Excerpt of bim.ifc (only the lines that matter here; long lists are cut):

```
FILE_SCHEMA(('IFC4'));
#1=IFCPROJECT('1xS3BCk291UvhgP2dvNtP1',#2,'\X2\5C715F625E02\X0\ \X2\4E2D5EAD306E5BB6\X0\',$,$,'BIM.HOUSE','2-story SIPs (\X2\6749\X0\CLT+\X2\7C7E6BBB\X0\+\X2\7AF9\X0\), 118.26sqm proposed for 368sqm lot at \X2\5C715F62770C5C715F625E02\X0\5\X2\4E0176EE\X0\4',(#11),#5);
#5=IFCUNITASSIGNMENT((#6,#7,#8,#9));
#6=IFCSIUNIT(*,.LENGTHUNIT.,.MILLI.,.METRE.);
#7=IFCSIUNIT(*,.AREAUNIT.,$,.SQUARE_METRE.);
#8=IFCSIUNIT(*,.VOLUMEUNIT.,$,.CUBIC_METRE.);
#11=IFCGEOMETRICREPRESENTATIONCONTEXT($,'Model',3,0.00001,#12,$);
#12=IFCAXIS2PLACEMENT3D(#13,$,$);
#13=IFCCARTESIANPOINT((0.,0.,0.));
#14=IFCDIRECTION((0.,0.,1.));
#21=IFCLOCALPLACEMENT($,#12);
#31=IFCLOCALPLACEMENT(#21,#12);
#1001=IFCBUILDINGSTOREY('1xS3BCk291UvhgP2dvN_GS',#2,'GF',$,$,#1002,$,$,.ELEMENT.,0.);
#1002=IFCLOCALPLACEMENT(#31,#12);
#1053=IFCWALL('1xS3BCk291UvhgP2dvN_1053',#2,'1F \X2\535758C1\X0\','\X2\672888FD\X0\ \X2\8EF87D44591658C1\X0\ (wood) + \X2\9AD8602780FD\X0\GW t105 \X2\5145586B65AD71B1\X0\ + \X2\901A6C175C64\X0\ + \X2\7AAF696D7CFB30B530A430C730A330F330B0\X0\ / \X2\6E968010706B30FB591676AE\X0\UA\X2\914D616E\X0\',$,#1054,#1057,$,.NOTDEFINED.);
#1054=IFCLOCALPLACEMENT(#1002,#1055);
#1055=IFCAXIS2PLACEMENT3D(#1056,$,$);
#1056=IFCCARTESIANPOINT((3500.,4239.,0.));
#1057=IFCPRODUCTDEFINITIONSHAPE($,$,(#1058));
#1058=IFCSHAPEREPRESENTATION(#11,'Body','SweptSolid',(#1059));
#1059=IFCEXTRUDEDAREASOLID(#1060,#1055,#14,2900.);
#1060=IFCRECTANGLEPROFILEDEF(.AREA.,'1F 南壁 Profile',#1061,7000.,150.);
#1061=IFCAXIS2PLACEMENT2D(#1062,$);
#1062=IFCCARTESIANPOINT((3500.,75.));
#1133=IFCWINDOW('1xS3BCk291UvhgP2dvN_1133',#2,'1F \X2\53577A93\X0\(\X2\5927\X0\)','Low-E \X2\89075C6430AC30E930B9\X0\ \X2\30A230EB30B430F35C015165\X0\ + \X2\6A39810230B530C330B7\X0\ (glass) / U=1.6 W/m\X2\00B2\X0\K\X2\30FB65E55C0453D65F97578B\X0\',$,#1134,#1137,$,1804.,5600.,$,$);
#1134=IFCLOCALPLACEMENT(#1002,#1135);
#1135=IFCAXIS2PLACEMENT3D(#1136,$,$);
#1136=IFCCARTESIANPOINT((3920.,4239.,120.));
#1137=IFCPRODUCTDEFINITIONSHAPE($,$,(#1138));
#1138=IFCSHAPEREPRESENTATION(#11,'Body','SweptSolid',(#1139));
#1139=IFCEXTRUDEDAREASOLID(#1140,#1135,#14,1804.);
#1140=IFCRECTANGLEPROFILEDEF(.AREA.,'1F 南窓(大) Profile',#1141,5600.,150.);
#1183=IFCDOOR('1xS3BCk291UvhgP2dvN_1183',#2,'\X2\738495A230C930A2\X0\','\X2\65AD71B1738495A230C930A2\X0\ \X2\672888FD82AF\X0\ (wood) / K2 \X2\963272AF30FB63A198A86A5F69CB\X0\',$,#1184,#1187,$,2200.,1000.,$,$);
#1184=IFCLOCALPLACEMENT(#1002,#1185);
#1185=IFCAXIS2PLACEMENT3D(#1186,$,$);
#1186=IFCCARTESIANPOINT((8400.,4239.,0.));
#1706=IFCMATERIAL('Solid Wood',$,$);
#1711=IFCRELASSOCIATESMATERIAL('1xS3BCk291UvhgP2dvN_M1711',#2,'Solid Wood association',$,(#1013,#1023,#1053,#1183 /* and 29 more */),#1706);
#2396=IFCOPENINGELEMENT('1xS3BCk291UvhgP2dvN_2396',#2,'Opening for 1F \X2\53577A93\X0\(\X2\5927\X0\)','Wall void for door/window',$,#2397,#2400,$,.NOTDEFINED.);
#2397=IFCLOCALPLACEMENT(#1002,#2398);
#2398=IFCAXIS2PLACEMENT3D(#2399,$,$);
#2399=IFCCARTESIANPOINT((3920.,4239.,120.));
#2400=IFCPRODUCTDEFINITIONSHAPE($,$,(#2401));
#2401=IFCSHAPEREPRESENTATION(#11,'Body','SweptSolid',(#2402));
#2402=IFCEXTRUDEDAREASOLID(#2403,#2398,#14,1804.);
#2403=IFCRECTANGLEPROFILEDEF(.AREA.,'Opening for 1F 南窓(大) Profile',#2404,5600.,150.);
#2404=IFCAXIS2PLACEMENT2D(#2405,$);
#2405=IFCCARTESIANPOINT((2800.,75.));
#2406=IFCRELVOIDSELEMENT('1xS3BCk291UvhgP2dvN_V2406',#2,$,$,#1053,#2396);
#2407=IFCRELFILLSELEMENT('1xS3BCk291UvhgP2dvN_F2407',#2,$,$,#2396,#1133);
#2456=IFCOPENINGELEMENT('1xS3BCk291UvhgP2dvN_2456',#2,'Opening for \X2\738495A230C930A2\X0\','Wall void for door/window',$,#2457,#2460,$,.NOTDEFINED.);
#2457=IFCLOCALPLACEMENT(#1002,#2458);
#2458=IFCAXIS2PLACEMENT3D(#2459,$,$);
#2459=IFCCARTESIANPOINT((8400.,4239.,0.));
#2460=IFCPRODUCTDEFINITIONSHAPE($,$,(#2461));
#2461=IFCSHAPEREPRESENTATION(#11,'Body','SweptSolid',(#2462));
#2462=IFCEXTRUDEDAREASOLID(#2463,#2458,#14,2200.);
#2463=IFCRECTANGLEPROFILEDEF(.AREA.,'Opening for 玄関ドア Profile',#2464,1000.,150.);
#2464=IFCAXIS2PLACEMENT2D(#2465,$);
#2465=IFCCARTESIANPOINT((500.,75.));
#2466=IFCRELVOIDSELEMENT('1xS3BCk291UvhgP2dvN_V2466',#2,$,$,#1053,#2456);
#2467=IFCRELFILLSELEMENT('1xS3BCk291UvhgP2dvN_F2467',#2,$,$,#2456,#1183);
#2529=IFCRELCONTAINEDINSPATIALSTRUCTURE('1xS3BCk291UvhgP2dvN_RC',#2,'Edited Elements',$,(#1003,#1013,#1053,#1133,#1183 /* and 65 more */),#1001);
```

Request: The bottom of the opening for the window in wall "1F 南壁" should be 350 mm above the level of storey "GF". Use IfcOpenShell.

```python
import numpy as np
import ifcopenshell
import ifcopenshell.api.geometry
import ifcopenshell.geom
import ifcopenshell.util.element
import ifcopenshell.util.placement
import ifcopenshell.util.shape
import ifcopenshell.util.unit

model = ifcopenshell.open("bim.ifc")
unit_scale = ifcopenshell.util.unit.calculate_unit_scale(model)

window = model.by_guid("1xS3BCk291UvhgP2dvN_1133")
opening = window.FillsVoids[0].RelatingOpeningElement
storey = ifcopenshell.util.element.get_container(window, ifc_class="IfcBuildingStorey")
level = ifcopenshell.util.placement.get_local_placement(storey.ObjectPlacement)[2, 3]

# The opening's origin need not be at the sill, so measure its lowest point.
shape = ifcopenshell.geom.create_shape(ifcopenshell.geom.settings(), opening)
bottom = ifcopenshell.util.shape.get_shape_bottom_elevation(shape, shape.geometry) / unit_scale
dz = level + 0.35 / unit_scale - bottom

shift = np.array([0.0, 0.0, dz])
# The window is not placed relative to its opening, so move both.
for product in (opening, window):
    matrix = ifcopenshell.util.placement.get_local_placement(product.ObjectPlacement)
    matrix[:3, 3] += shift
    ifcopenshell.api.geometry.edit_object_placement(model, product=product, matrix=matrix, is_si=False)

print(f"moved by {dz * unit_scale:+.3f} m")

model.write("bim_rev.ifc")
```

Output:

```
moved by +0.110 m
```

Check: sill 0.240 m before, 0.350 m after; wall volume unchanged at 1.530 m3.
